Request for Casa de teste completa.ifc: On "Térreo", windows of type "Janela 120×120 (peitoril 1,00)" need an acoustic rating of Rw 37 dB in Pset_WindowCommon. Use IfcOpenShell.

First a look at what the model holds.

```python
import ifcopenshell
import ifcopenshell.util.element

model = ifcopenshell.open("Casa de teste completa.ifc")
print(model.schema)
storey = next(s for s in model.by_type("IfcBuildingStorey") if s.Name == "Térreo")
windows = [e for e in ifcopenshell.util.element.get_decomposition(storey) if e.is_a("IfcWindow")]
seen = {}
for e in windows:
    element_type = ifcopenshell.util.element.get_type(e)
    key = (element_type.Name if element_type != e and element_type else None, ifcopenshell.util.element.get_pset(e, "Pset_WindowCommon", "AcousticRating"))
    seen[key] = seen.get(key, 0) + 1
for (name, value), count in sorted(seen.items(), key=str):
    print(count, "x", name, "|", value)
```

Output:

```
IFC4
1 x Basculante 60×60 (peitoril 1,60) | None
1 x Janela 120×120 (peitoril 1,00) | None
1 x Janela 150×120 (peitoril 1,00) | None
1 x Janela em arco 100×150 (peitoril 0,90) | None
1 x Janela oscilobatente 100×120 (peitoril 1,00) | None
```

```python
import ifcopenshell
import ifcopenshell.api.pset
import ifcopenshell.util.element

model = ifcopenshell.open("Casa de teste completa.ifc")

storey = next(s for s in model.by_type("IfcBuildingStorey") if s.Name == "Térreo")
windows = [e for e in ifcopenshell.util.element.get_decomposition(storey) if e.is_a("IfcWindow")]

count = 0
for e in windows:
    element_type = ifcopenshell.util.element.get_type(e)
    if element_type in (None, e) or element_type.Name != "Janela 120×120 (peitoril 1,00)":
        continue
    # add_pset returns the element's existing set when there is one.
    pset = ifcopenshell.api.pset.add_pset(model, product=e, name="Pset_WindowCommon")
    ifcopenshell.api.pset.edit_pset(model, pset=pset, properties={"AcousticRating": "Rw 37 dB"})
    count += 1

print(count, "windows updated")

model.write("Casa de teste completa-out.ifc")
```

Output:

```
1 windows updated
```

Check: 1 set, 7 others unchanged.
